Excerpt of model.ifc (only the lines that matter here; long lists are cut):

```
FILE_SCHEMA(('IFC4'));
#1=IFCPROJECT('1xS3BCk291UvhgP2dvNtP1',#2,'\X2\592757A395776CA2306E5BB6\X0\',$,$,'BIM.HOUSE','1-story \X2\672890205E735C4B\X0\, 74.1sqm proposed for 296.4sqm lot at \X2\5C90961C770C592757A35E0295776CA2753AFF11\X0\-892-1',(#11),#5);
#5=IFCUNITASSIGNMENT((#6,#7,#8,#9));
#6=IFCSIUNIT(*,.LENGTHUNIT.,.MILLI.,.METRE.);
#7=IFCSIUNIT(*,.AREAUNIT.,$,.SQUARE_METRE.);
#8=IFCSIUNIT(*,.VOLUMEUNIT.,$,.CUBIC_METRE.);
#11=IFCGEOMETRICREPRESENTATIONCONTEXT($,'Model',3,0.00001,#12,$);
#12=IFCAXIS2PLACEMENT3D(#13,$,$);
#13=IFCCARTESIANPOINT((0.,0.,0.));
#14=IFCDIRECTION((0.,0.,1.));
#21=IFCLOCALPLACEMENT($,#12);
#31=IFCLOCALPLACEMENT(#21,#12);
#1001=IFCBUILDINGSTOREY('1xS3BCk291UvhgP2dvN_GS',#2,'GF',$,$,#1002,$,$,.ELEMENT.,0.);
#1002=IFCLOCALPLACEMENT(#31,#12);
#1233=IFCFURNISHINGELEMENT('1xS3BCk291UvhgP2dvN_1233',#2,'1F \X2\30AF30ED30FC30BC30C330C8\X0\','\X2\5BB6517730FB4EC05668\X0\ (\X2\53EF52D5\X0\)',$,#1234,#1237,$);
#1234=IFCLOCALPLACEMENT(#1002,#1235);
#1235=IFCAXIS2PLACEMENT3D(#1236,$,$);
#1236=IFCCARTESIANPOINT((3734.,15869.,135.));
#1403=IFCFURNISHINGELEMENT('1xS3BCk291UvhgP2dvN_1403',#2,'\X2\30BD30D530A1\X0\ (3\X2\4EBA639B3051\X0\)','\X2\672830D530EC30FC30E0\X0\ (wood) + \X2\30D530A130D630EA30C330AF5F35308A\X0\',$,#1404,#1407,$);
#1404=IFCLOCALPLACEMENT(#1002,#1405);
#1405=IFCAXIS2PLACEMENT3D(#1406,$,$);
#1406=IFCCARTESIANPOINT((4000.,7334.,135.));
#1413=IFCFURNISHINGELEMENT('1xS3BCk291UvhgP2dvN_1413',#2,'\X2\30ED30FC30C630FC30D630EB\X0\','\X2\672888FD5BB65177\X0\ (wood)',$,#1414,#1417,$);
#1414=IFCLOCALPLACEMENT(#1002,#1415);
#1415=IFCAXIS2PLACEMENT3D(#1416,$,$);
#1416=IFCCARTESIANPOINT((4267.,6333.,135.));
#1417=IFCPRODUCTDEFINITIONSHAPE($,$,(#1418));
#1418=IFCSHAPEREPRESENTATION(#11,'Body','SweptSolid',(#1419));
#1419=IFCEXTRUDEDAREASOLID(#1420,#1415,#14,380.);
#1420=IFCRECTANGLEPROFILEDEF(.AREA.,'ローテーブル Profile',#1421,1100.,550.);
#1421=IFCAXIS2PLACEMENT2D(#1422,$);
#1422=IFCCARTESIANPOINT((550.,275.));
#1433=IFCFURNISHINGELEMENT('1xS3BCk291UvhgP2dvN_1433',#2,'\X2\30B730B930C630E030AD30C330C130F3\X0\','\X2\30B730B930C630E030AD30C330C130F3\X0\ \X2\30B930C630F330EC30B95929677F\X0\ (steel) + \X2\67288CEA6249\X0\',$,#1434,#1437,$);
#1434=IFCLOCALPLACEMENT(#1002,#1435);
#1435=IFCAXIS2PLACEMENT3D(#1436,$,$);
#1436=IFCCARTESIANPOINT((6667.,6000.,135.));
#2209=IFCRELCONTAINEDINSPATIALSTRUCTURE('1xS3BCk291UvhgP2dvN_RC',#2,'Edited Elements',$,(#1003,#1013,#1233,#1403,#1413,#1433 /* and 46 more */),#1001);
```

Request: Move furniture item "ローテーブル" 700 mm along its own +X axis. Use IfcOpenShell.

```python
import ifcopenshell
import ifcopenshell.api.geometry
import ifcopenshell.util.placement
import ifcopenshell.util.unit

model = ifcopenshell.open("model.ifc")
unit_scale = ifcopenshell.util.unit.calculate_unit_scale(model)

item = model.by_guid("1xS3BCk291UvhgP2dvN_1413")
matrix = ifcopenshell.util.placement.get_local_placement(item.ObjectPlacement)
matrix[:3, 3] += matrix[:3, 0] * 0.7 / unit_scale
ifcopenshell.api.geometry.edit_object_placement(model, product=item, matrix=matrix, is_si=False)

print(ifcopenshell.util.placement.get_local_placement(item.ObjectPlacement).round(3) + 0.0)

model.write("model_updated.ifc")
```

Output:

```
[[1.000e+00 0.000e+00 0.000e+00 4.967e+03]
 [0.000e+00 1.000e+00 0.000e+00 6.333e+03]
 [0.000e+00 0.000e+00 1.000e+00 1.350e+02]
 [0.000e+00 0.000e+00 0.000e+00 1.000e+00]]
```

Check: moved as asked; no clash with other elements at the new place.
